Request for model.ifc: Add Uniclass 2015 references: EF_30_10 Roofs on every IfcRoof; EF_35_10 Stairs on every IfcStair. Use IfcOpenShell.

First a look at what the model holds.

```python
import ifcopenshell

model = ifcopenshell.open("model.ifc")
print(model.schema)
print("classifications:", [c.Name for c in model.by_type("IfcClassification")])
for ifc_class in ("IfcDoor", "IfcRoof", "IfcStair", "IfcWall", "IfcWindow"):
    print(ifc_class, len(model.by_type(ifc_class)))
```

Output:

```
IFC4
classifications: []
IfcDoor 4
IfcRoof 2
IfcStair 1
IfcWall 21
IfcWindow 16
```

```python
import ifcopenshell
import ifcopenshell.api.classification

model = ifcopenshell.open("model.ifc")

system = ifcopenshell.api.classification.add_classification(model, classification="Uniclass 2015")

codes = {
    "IfcRoof": ("EF_30_10", "Roofs"),
    "IfcStair": ("EF_35_10", "Stairs"),
}
for ifc_class, (code, name) in codes.items():
    products = model.by_type(ifc_class)
    ifcopenshell.api.classification.add_reference(
        model, products=products, classification=system, identification=code, name=name
    )
    print(code, len(products))

model.write("model_edited.ifc")
```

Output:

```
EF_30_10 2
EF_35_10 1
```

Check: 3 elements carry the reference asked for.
